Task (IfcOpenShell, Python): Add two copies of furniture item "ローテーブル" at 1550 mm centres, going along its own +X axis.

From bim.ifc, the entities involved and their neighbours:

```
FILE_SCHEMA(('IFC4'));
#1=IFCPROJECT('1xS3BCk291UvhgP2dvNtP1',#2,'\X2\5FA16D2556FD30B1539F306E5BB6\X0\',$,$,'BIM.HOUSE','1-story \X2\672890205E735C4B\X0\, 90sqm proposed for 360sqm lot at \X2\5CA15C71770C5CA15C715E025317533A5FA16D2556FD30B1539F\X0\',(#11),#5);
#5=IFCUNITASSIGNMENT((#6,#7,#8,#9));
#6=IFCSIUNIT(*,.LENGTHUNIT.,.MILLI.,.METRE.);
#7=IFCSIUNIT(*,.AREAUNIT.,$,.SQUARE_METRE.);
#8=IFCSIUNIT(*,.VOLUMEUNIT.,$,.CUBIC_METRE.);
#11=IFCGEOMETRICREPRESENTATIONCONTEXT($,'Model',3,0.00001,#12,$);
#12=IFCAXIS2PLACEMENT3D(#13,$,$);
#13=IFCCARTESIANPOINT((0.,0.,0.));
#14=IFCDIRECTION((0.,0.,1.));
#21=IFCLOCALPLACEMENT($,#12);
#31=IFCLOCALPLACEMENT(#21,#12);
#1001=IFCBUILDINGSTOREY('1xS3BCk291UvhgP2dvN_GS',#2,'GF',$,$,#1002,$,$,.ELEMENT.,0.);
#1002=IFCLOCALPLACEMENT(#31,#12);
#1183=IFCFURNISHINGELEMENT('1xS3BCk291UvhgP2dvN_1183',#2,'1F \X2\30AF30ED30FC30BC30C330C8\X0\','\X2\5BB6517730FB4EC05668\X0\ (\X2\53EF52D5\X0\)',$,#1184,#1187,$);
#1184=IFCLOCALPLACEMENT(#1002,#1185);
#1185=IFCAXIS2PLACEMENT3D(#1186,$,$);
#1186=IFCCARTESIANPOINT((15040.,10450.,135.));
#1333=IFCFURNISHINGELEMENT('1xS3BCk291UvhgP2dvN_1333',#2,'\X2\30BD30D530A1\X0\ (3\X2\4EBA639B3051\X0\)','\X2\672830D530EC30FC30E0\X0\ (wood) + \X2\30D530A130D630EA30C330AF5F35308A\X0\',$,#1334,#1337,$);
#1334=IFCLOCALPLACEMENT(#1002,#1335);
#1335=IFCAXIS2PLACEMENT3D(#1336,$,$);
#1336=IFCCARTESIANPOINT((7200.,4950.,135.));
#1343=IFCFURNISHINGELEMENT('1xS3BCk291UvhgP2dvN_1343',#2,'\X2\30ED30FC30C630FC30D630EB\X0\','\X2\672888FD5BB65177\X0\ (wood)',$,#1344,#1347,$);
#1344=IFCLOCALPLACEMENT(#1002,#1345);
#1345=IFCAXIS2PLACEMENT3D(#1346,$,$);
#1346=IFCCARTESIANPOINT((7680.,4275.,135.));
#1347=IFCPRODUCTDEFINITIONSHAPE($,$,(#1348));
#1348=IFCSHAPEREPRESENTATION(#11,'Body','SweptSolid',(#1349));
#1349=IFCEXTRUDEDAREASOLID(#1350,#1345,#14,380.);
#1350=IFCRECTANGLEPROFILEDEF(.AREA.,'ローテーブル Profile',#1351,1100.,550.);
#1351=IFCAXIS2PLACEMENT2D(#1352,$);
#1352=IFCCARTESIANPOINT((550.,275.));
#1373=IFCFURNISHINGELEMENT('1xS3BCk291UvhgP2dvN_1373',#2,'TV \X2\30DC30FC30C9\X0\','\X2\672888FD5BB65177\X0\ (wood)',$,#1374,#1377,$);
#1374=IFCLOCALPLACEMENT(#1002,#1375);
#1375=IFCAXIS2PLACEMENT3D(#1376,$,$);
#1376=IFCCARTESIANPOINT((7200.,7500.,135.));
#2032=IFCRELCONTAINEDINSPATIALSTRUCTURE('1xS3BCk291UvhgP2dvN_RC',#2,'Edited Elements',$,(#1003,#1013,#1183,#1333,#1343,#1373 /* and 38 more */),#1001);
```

```python
import ifcopenshell
import ifcopenshell.api.geometry
import ifcopenshell.api.root
import ifcopenshell.util.element
import ifcopenshell.util.placement
import ifcopenshell.util.unit

model = ifcopenshell.open("bim.ifc")
unit_scale = ifcopenshell.util.unit.calculate_unit_scale(model)


def reuse_history(source, copy):
    """copy_class also copies each property set's owner history, people and application; keep the originals."""
    for rel in copy.IsDefinedBy:
        if rel.is_a("IfcRelDefinesByProperties") and (history := rel.RelatingPropertyDefinition.OwnerHistory):
            rel.RelatingPropertyDefinition.OwnerHistory = source.OwnerHistory
            ifcopenshell.util.element.remove_deep2(model, history)


source = model.by_id(1343)
base = ifcopenshell.util.placement.get_local_placement(source.ObjectPlacement)
step = base[:3, 0] * 1.55 / unit_scale

for i in range(1, 3):
    copy = ifcopenshell.api.root.copy_class(model, product=source)
    copy.Representation = ifcopenshell.util.element.copy_deep(
        model, source.Representation, exclude=["IfcGeometricRepresentationContext", "IfcRepresentationMap"]
    )
    reuse_history(source, copy)
    matrix = base.copy()
    matrix[:3, 3] += i * step
    print("added at", matrix[:3, 3].round(3) + 0.0)
    ifcopenshell.api.geometry.edit_object_placement(model, product=copy, matrix=matrix, is_si=False)

model.write("bim_edited.ifc")
```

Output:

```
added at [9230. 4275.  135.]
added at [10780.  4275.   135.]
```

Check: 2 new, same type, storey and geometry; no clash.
